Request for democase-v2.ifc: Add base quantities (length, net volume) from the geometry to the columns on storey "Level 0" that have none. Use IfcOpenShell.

First a look at what the model holds.

```python
import ifcopenshell
import ifcopenshell.util.element
import ifcopenshell.util.unit

model = ifcopenshell.open("democase-v2.ifc")
print(model.schema)
for unit_type in ("LENGTHUNIT", "AREAUNIT", "VOLUMEUNIT"):
    print(unit_type, ifcopenshell.util.unit.calculate_unit_scale(model, unit_type))
storey = next(s for s in model.by_type("IfcBuildingStorey") if s.Name == "Level 0")
columns = [e for e in ifcopenshell.util.element.get_decomposition(storey) if e.is_a("IfcColumn")]
for e in sorted(columns, key=lambda e: e.id()):
    print(e.id(), e.is_a(), e.Name, list(ifcopenshell.util.element.get_psets(e, qtos_only=True)), sep=" | ")
```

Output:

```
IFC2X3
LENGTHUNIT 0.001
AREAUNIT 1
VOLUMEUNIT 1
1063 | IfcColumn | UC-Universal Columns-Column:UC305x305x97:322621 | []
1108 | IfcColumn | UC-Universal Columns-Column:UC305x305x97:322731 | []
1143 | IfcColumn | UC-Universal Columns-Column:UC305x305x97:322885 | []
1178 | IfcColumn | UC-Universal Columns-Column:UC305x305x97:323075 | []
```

```python
import ifcopenshell
import ifcopenshell.api.pset
import ifcopenshell.geom
import ifcopenshell.util.element
import ifcopenshell.util.shape
import ifcopenshell.util.unit

model = ifcopenshell.open("democase-v2.ifc")
unit_scale = ifcopenshell.util.unit.calculate_unit_scale(model)
volume_scale = ifcopenshell.util.unit.calculate_unit_scale(model, "VOLUMEUNIT")
settings = ifcopenshell.geom.settings()

storey = next(s for s in model.by_type("IfcBuildingStorey") if s.Name == "Level 0")
columns = [e for e in ifcopenshell.util.element.get_decomposition(storey) if e.is_a("IfcColumn")]

for e in sorted(columns, key=lambda e: e.id()):
    if ifcopenshell.util.element.get_psets(e, qtos_only=True, should_inherit=False):
        continue
    # Geometry comes back in metres, in the element's own axes.
    shape = ifcopenshell.geom.create_shape(settings, e)
    values = {
        "Length": ifcopenshell.util.shape.get_z(shape.geometry) / unit_scale,
        "NetVolume": ifcopenshell.util.shape.get_volume(shape.geometry) / volume_scale,
    }
    qto = ifcopenshell.api.pset.add_qto(model, product=e, name="BaseQuantities")
    ifcopenshell.api.pset.edit_qto(model, qto=qto, properties=values)
    print(e.id(), {k: round(v, 3) for k, v in values.items()})

model.write("democase-v2_v2.ifc")
```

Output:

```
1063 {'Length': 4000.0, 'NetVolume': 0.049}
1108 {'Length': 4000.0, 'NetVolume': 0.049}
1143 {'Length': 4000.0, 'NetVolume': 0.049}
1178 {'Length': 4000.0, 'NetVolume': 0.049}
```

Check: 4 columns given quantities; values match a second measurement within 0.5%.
